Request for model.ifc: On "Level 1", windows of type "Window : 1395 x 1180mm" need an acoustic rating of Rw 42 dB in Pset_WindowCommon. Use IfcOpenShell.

First a look at what the model holds.

```python
import ifcopenshell
import ifcopenshell.util.element

model = ifcopenshell.open("model.ifc")
print(model.schema)
storey = next(s for s in model.by_type("IfcBuildingStorey") if s.Name == "Level 1")
windows = [e for e in ifcopenshell.util.element.get_decomposition(storey) if e.is_a("IfcWindow")]
seen = {}
for e in windows:
    element_type = ifcopenshell.util.element.get_type(e)
    key = (element_type.Name if element_type != e and element_type else None, ifcopenshell.util.element.get_pset(e, "Pset_WindowCommon", "AcousticRating"))
    seen[key] = seen.get(key, 0) + 1
for (name, value), count in sorted(seen.items(), key=str):
    print(count, "x", name, "|", value)
```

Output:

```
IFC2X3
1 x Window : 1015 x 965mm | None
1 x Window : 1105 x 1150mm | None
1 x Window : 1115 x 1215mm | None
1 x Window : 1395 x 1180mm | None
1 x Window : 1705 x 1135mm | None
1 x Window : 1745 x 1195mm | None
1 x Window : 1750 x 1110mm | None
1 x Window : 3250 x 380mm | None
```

```python
import ifcopenshell
import ifcopenshell.api.pset
import ifcopenshell.util.element

model = ifcopenshell.open("model.ifc")

storey = next(s for s in model.by_type("IfcBuildingStorey") if s.Name == "Level 1")
windows = [e for e in ifcopenshell.util.element.get_decomposition(storey) if e.is_a("IfcWindow")]

count = 0
for e in windows:
    element_type = ifcopenshell.util.element.get_type(e)
    if element_type in (None, e) or element_type.Name != "Window : 1395 x 1180mm":
        continue
    # add_pset returns the element's existing set when there is one.
    pset = ifcopenshell.api.pset.add_pset(model, product=e, name="Pset_WindowCommon")
    ifcopenshell.api.pset.edit_pset(model, pset=pset, properties={"AcousticRating": "Rw 42 dB"})
    count += 1

print(count, "windows updated")

model.write("model_v2.ifc")
```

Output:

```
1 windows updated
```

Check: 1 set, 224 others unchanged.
